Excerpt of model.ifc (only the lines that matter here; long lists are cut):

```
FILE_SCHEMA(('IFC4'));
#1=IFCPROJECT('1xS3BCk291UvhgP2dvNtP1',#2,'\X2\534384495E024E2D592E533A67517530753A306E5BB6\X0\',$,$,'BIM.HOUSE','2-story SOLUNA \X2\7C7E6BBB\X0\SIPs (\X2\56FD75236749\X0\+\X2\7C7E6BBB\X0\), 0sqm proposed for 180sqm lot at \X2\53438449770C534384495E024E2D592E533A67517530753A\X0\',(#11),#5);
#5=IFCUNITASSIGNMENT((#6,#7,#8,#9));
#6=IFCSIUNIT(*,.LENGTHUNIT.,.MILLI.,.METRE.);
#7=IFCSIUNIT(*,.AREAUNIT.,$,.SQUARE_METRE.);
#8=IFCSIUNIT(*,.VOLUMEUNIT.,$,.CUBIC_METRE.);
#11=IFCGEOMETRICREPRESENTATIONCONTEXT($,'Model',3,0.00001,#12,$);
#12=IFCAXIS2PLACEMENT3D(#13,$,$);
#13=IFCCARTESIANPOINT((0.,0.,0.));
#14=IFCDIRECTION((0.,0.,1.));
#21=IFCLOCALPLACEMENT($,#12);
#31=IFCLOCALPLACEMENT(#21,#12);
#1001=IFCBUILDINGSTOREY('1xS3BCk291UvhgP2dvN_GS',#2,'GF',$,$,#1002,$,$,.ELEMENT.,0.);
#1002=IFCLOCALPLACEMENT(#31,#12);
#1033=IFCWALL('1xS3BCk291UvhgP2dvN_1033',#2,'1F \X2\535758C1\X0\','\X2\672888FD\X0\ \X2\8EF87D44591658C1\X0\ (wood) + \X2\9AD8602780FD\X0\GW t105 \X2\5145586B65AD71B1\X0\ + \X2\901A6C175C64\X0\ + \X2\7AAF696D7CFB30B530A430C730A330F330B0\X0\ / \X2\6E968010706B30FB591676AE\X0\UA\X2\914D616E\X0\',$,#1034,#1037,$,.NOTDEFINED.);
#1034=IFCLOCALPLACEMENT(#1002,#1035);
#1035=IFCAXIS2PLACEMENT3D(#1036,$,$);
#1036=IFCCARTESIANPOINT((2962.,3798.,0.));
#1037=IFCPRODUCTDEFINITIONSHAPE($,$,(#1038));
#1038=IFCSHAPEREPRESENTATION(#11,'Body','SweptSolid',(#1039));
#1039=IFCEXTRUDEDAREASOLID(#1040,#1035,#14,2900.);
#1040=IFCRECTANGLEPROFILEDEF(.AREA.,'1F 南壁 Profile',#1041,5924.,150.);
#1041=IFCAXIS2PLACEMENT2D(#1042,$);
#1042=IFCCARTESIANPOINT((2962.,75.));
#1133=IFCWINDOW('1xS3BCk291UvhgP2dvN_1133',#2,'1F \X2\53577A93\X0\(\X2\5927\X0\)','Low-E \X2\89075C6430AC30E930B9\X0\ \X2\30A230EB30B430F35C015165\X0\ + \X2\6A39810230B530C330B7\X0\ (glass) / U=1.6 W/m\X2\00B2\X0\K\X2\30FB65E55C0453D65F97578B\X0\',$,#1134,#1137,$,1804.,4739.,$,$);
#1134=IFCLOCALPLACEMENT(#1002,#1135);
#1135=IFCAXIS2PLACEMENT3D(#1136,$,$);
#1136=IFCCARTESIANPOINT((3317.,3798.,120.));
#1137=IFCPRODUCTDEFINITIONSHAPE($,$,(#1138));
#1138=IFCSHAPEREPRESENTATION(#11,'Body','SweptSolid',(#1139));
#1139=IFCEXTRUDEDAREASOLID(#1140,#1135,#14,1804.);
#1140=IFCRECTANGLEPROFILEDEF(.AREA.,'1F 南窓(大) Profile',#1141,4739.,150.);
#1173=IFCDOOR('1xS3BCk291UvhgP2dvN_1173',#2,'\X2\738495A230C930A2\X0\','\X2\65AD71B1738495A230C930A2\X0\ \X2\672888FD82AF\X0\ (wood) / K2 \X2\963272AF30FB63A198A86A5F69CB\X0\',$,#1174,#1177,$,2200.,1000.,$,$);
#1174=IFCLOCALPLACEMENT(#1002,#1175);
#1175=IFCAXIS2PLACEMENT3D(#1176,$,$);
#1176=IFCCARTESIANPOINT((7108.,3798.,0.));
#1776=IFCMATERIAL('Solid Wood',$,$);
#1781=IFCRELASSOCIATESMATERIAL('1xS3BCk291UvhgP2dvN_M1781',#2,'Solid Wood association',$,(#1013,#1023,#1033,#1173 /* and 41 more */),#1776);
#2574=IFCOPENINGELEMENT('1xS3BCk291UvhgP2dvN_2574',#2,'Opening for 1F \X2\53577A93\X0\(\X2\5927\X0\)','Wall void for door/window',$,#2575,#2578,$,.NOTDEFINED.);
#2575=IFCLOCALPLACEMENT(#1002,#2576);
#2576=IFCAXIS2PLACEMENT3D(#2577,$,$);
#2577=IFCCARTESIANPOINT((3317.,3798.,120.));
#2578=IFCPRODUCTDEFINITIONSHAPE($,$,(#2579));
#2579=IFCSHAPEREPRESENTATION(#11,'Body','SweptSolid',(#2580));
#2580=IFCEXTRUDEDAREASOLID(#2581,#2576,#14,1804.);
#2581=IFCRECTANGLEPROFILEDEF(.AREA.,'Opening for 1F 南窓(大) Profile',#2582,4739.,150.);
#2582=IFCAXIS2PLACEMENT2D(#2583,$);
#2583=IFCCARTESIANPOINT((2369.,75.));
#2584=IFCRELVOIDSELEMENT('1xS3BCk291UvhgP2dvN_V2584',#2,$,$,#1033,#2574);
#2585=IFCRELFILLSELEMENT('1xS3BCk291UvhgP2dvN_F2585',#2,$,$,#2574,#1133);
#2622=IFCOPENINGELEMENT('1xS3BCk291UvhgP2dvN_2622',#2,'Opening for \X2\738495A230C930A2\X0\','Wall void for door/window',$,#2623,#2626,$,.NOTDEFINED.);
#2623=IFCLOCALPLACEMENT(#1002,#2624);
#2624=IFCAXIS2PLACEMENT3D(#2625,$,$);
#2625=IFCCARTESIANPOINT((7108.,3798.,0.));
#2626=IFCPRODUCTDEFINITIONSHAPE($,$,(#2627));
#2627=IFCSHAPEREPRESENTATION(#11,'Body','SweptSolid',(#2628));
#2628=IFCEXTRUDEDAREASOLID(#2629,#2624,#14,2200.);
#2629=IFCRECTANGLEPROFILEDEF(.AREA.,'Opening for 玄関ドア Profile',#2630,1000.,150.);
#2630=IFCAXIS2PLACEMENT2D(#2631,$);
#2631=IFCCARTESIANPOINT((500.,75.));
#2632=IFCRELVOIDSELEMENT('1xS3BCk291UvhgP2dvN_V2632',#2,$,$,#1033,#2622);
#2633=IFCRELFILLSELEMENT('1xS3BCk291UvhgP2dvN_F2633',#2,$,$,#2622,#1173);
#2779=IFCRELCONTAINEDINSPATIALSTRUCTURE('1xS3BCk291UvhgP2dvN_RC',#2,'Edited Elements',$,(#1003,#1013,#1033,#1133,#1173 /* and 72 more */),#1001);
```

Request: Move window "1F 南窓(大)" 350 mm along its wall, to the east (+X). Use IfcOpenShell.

```python
import ifcopenshell
import ifcopenshell.api.geometry
import ifcopenshell.util.placement
import ifcopenshell.util.unit

model = ifcopenshell.open("model.ifc")
unit_scale = ifcopenshell.util.unit.calculate_unit_scale(model)

window = model.by_guid("1xS3BCk291UvhgP2dvN_1133")
opening = window.FillsVoids[0].RelatingOpeningElement
wall = opening.VoidsElements[0].RelatingBuildingElement

wall_matrix = ifcopenshell.util.placement.get_local_placement(wall.ObjectPlacement)
shift = wall_matrix[:3, 0] * 0.35 / unit_scale
before = ifcopenshell.util.placement.get_local_placement(window.ObjectPlacement)[:3, 3].copy()

# The window is not placed relative to its opening, so move both.
for product in (opening, window):
    matrix = ifcopenshell.util.placement.get_local_placement(product.ObjectPlacement)
    matrix[:3, 3] += shift
    ifcopenshell.api.geometry.edit_object_placement(model, product=product, matrix=matrix, is_si=False)

after = ifcopenshell.util.placement.get_local_placement(window.ObjectPlacement)[:3, 3]
print("window moved by", (after - before).round(3) + 0.0)

model.write("model_edited.ifc")
```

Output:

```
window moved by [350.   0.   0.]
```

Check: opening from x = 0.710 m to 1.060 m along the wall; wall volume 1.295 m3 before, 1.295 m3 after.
